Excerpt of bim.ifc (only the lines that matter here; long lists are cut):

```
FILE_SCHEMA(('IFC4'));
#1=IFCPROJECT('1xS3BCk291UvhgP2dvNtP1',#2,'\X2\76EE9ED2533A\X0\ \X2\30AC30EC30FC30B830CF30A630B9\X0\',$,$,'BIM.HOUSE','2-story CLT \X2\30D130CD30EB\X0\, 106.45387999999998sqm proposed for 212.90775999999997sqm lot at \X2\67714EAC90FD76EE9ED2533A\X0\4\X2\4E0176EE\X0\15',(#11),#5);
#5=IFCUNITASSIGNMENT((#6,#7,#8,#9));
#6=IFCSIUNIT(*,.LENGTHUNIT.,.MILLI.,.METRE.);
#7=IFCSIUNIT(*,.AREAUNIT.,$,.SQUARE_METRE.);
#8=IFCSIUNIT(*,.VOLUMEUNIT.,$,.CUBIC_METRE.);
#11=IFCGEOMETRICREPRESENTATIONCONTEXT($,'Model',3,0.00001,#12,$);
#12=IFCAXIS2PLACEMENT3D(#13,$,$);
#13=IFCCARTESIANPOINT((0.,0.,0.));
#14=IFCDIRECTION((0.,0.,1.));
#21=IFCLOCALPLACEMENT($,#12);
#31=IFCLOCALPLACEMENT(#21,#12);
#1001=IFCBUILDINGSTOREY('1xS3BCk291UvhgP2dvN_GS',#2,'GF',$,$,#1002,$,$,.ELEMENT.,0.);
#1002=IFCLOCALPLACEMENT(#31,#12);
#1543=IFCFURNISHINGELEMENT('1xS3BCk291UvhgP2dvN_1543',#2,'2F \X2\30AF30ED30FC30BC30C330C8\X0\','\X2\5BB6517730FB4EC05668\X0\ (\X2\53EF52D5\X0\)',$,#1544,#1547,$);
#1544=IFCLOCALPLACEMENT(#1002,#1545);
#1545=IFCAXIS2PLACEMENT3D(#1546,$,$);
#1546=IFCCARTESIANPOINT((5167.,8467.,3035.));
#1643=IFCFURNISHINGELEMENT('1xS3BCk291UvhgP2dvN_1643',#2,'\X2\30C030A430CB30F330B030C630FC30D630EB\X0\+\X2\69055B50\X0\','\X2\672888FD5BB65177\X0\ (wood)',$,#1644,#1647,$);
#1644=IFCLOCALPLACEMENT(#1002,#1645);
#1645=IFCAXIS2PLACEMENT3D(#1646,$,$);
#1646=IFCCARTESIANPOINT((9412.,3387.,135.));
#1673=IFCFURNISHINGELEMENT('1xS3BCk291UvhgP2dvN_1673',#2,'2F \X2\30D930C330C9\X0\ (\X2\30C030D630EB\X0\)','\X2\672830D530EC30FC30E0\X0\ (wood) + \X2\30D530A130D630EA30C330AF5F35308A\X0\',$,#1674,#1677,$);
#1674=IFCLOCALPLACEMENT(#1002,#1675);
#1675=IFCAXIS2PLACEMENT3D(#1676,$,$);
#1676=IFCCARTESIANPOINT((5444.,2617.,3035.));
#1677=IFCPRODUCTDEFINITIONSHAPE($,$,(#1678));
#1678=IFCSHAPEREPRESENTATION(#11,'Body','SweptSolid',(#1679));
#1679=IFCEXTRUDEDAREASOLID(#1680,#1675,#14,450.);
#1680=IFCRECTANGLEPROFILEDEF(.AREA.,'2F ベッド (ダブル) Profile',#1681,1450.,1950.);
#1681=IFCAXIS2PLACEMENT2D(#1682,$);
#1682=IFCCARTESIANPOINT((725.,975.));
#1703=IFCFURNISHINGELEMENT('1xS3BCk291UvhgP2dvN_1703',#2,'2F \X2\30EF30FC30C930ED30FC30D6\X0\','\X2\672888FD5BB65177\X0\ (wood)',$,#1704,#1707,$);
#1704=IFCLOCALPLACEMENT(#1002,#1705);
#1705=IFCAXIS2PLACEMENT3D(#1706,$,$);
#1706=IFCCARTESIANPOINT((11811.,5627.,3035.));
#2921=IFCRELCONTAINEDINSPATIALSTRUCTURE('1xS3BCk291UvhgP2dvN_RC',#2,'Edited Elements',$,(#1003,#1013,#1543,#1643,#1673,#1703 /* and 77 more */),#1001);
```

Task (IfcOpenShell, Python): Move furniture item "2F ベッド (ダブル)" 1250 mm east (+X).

```python
import ifcopenshell
import ifcopenshell.api.geometry
import ifcopenshell.util.placement

model = ifcopenshell.open("bim.ifc")

item = model.by_id(1673)
matrix = ifcopenshell.util.placement.get_local_placement(item.ObjectPlacement)
matrix[0, 3] += 1250.0
ifcopenshell.api.geometry.edit_object_placement(model, product=item, matrix=matrix, is_si=False)

print(ifcopenshell.util.placement.get_local_placement(item.ObjectPlacement).round(3) + 0.0)

model.write("bim_v2.ifc")
```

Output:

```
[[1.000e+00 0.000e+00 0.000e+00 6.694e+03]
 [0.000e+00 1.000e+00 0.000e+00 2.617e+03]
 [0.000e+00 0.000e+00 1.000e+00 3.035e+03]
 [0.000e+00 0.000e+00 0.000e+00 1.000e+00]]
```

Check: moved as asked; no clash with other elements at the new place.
